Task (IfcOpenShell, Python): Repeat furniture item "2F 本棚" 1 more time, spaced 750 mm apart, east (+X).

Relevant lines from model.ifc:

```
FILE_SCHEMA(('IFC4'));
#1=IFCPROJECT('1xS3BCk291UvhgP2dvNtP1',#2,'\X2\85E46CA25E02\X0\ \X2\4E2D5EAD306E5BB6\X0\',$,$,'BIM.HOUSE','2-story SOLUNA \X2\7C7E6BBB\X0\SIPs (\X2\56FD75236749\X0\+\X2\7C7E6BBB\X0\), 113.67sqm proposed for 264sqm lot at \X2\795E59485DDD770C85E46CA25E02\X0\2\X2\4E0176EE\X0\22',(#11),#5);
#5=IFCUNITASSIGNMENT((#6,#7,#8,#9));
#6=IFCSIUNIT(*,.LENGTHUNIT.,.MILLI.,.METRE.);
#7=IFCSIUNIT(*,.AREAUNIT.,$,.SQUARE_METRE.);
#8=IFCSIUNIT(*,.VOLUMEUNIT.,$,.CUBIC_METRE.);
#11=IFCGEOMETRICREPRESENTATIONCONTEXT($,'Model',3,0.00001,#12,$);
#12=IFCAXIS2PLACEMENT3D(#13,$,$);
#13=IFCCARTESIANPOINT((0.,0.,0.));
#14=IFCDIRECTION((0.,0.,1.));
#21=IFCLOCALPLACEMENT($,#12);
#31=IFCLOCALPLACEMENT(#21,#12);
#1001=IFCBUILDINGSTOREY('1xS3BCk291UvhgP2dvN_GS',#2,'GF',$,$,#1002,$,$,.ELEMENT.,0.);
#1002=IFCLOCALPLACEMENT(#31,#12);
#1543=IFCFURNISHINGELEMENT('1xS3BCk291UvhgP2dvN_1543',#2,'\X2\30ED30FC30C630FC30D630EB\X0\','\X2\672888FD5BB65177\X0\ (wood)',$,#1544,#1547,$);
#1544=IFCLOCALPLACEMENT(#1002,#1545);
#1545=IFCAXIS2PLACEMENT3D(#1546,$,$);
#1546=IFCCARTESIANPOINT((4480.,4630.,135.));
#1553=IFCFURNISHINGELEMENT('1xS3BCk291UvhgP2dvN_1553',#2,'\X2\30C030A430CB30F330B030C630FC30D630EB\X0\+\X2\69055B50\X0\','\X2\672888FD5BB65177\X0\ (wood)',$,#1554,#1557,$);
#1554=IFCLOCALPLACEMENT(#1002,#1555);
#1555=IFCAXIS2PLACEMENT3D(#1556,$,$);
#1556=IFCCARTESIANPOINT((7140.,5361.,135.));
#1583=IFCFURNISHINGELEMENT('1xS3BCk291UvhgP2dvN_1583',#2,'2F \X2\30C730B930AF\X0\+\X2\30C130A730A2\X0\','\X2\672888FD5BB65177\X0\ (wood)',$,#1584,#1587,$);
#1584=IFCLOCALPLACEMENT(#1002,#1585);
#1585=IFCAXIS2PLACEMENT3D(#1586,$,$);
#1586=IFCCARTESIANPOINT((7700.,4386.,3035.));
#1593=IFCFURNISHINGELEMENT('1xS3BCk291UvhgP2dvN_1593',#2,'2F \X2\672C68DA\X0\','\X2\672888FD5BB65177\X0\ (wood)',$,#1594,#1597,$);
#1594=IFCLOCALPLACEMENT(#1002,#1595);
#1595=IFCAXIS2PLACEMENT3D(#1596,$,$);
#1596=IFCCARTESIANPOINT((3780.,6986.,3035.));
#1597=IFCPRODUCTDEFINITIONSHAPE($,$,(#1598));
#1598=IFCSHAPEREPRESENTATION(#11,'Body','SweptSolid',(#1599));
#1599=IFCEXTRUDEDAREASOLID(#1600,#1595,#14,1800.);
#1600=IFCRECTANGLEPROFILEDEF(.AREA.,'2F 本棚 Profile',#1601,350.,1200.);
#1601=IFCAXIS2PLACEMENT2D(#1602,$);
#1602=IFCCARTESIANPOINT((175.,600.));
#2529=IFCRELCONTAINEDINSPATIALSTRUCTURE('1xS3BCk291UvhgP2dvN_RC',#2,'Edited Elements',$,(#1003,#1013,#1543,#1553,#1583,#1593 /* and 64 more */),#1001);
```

```python
import numpy as np
import ifcopenshell
import ifcopenshell.api.geometry
import ifcopenshell.api.root
import ifcopenshell.util.element
import ifcopenshell.util.placement

model = ifcopenshell.open("model.ifc")


def reuse_history(source, copy):
    """copy_class also copies each property set's owner history, people and application; keep the originals."""
    for rel in copy.IsDefinedBy:
        if rel.is_a("IfcRelDefinesByProperties") and (history := rel.RelatingPropertyDefinition.OwnerHistory):
            rel.RelatingPropertyDefinition.OwnerHistory = source.OwnerHistory
            ifcopenshell.util.element.remove_deep2(model, history)


source = model.by_guid("1xS3BCk291UvhgP2dvN_1593")
base = ifcopenshell.util.placement.get_local_placement(source.ObjectPlacement)
step = np.array([1.0, 0.0, 0.0]) * 750.0

for i in range(1, 2):
    copy = ifcopenshell.api.root.copy_class(model, product=source)
    copy.Representation = ifcopenshell.util.element.copy_deep(
        model, source.Representation, exclude=["IfcGeometricRepresentationContext", "IfcRepresentationMap"]
    )
    reuse_history(source, copy)
    matrix = base.copy()
    matrix[:3, 3] += i * step
    print("added at", matrix[:3, 3].round(3) + 0.0)
    ifcopenshell.api.geometry.edit_object_placement(model, product=copy, matrix=matrix, is_si=False)

model.write("model_edited.ifc")
```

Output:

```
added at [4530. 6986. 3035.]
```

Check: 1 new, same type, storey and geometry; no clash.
